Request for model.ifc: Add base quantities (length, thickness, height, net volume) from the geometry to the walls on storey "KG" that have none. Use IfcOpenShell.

First a look at what the model holds.

```python
import ifcopenshell
import ifcopenshell.util.element
import ifcopenshell.util.unit

model = ifcopenshell.open("model.ifc")
print(model.schema)
for unit_type in ("LENGTHUNIT", "AREAUNIT", "VOLUMEUNIT"):
    print(unit_type, ifcopenshell.util.unit.calculate_unit_scale(model, unit_type))
storey = next(s for s in model.by_type("IfcBuildingStorey") if s.Name == "KG")
walls = [e for e in ifcopenshell.util.element.get_decomposition(storey) if e.is_a("IfcWall")]
for e in sorted(walls, key=lambda e: e.id()):
    print(e.id(), e.is_a(), e.Name, list(ifcopenshell.util.element.get_psets(e, qtos_only=True)), sep=" | ")
```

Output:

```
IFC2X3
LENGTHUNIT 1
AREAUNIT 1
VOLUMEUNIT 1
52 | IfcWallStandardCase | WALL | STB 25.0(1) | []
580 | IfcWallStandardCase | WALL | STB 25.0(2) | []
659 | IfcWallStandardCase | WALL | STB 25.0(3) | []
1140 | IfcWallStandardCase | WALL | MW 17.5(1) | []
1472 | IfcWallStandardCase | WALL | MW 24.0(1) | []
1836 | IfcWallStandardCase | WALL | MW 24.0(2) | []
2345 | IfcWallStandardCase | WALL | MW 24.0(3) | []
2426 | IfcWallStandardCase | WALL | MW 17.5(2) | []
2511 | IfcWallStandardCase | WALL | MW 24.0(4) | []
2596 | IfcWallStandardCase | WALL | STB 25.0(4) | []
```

```python
import ifcopenshell
import ifcopenshell.api.pset
import ifcopenshell.geom
import ifcopenshell.util.element
import ifcopenshell.util.shape
import ifcopenshell.util.unit

model = ifcopenshell.open("model.ifc")
unit_scale = ifcopenshell.util.unit.calculate_unit_scale(model)
volume_scale = ifcopenshell.util.unit.calculate_unit_scale(model, "VOLUMEUNIT")
settings = ifcopenshell.geom.settings()

storey = next(s for s in model.by_type("IfcBuildingStorey") if s.Name == "KG")
walls = [e for e in ifcopenshell.util.element.get_decomposition(storey) if e.is_a("IfcWall")]

for e in sorted(walls, key=lambda e: e.id()):
    if ifcopenshell.util.element.get_psets(e, qtos_only=True, should_inherit=False):
        continue
    # Geometry comes back in metres, in the element's own axes.
    shape = ifcopenshell.geom.create_shape(settings, e)
    values = {
        "Length": ifcopenshell.util.shape.get_x(shape.geometry) / unit_scale,
        "Width": ifcopenshell.util.shape.get_y(shape.geometry) / unit_scale,
        "Height": ifcopenshell.util.shape.get_z(shape.geometry) / unit_scale,
        "NetVolume": ifcopenshell.util.shape.get_volume(shape.geometry) / volume_scale,
    }
    qto = ifcopenshell.api.pset.add_qto(model, product=e, name="BaseQuantities")
    ifcopenshell.api.pset.edit_qto(model, qto=qto, properties=values)
    print(e.id(), {k: round(v, 3) for k, v in values.items()})

model.write("model_updated.ifc")
```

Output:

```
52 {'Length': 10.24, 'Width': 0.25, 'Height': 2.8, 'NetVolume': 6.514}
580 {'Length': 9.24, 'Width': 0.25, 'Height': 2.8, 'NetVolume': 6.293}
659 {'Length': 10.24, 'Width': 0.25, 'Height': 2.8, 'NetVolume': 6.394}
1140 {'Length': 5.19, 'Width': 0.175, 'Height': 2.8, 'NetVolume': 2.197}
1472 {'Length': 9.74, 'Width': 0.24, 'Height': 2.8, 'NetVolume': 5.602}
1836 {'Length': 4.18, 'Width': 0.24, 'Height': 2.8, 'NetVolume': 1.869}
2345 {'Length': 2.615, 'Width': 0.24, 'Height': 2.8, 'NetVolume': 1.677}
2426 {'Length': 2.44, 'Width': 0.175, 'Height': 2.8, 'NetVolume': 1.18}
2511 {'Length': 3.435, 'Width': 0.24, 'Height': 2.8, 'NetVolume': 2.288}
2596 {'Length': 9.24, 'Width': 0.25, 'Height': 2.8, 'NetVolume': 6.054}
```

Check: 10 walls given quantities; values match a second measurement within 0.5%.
